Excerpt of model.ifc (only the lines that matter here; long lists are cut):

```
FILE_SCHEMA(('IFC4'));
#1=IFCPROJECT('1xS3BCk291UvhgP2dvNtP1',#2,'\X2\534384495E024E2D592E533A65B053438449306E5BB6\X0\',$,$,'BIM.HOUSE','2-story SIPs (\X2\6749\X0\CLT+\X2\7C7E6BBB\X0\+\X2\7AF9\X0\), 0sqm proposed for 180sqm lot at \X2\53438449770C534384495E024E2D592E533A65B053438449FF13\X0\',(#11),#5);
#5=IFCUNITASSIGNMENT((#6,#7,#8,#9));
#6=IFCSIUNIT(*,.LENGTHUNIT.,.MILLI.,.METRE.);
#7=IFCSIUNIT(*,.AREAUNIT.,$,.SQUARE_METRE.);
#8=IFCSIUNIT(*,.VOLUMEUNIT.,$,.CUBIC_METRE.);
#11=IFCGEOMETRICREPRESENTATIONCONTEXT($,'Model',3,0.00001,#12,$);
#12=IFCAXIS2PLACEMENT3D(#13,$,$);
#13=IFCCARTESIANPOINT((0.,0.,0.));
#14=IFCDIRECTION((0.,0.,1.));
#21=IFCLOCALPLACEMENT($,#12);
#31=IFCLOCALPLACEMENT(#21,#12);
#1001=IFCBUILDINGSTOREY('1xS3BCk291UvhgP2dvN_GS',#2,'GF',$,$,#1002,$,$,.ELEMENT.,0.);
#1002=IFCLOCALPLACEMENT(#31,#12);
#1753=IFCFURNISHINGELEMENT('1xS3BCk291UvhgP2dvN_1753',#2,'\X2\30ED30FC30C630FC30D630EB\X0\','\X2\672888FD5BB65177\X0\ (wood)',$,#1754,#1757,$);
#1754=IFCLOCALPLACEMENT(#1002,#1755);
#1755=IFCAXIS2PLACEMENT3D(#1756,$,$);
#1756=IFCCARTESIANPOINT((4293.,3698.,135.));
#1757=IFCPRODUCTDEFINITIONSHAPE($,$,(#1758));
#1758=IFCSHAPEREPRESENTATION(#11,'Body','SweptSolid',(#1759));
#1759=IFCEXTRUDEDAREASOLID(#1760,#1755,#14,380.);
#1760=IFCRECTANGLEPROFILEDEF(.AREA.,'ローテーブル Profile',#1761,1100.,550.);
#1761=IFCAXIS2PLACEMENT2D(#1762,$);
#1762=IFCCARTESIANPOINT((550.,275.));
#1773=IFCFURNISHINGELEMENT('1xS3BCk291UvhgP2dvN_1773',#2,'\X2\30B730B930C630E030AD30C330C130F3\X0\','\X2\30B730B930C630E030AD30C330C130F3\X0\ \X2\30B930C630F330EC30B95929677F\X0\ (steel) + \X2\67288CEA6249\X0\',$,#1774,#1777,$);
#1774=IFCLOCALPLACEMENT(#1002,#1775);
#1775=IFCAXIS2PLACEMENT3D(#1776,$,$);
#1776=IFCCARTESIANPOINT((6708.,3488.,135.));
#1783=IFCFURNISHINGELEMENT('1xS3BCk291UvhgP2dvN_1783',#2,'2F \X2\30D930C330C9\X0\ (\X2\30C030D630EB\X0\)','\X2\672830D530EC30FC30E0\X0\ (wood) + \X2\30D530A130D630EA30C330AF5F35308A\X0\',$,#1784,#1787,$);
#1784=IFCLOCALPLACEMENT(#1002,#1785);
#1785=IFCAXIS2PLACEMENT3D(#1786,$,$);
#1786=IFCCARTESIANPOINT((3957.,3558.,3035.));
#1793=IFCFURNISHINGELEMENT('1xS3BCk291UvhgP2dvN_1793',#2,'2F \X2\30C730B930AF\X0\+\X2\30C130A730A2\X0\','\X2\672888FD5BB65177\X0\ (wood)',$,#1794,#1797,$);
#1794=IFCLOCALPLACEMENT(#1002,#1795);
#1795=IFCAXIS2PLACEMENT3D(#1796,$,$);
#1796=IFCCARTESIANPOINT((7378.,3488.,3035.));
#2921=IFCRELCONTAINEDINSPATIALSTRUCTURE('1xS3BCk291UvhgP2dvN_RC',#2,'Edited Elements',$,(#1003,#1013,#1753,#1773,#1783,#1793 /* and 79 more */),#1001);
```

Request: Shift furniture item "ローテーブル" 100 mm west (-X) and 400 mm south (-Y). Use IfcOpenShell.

```python
import ifcopenshell
import ifcopenshell.api.geometry
import ifcopenshell.util.placement
import ifcopenshell.util.unit

model = ifcopenshell.open("model.ifc")
unit_scale = ifcopenshell.util.unit.calculate_unit_scale(model)

item = model.by_guid("1xS3BCk291UvhgP2dvN_1753")
matrix = ifcopenshell.util.placement.get_local_placement(item.ObjectPlacement)
matrix[0, 3] -= 0.1 / unit_scale
matrix[1, 3] -= 0.4 / unit_scale
ifcopenshell.api.geometry.edit_object_placement(model, product=item, matrix=matrix, is_si=False)

print(ifcopenshell.util.placement.get_local_placement(item.ObjectPlacement).round(3) + 0.0)

model.write("model_v2.ifc")
```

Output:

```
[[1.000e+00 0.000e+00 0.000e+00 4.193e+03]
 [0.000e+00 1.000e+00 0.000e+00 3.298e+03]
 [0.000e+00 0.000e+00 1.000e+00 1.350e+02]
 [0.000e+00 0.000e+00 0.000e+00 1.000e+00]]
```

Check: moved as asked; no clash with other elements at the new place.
